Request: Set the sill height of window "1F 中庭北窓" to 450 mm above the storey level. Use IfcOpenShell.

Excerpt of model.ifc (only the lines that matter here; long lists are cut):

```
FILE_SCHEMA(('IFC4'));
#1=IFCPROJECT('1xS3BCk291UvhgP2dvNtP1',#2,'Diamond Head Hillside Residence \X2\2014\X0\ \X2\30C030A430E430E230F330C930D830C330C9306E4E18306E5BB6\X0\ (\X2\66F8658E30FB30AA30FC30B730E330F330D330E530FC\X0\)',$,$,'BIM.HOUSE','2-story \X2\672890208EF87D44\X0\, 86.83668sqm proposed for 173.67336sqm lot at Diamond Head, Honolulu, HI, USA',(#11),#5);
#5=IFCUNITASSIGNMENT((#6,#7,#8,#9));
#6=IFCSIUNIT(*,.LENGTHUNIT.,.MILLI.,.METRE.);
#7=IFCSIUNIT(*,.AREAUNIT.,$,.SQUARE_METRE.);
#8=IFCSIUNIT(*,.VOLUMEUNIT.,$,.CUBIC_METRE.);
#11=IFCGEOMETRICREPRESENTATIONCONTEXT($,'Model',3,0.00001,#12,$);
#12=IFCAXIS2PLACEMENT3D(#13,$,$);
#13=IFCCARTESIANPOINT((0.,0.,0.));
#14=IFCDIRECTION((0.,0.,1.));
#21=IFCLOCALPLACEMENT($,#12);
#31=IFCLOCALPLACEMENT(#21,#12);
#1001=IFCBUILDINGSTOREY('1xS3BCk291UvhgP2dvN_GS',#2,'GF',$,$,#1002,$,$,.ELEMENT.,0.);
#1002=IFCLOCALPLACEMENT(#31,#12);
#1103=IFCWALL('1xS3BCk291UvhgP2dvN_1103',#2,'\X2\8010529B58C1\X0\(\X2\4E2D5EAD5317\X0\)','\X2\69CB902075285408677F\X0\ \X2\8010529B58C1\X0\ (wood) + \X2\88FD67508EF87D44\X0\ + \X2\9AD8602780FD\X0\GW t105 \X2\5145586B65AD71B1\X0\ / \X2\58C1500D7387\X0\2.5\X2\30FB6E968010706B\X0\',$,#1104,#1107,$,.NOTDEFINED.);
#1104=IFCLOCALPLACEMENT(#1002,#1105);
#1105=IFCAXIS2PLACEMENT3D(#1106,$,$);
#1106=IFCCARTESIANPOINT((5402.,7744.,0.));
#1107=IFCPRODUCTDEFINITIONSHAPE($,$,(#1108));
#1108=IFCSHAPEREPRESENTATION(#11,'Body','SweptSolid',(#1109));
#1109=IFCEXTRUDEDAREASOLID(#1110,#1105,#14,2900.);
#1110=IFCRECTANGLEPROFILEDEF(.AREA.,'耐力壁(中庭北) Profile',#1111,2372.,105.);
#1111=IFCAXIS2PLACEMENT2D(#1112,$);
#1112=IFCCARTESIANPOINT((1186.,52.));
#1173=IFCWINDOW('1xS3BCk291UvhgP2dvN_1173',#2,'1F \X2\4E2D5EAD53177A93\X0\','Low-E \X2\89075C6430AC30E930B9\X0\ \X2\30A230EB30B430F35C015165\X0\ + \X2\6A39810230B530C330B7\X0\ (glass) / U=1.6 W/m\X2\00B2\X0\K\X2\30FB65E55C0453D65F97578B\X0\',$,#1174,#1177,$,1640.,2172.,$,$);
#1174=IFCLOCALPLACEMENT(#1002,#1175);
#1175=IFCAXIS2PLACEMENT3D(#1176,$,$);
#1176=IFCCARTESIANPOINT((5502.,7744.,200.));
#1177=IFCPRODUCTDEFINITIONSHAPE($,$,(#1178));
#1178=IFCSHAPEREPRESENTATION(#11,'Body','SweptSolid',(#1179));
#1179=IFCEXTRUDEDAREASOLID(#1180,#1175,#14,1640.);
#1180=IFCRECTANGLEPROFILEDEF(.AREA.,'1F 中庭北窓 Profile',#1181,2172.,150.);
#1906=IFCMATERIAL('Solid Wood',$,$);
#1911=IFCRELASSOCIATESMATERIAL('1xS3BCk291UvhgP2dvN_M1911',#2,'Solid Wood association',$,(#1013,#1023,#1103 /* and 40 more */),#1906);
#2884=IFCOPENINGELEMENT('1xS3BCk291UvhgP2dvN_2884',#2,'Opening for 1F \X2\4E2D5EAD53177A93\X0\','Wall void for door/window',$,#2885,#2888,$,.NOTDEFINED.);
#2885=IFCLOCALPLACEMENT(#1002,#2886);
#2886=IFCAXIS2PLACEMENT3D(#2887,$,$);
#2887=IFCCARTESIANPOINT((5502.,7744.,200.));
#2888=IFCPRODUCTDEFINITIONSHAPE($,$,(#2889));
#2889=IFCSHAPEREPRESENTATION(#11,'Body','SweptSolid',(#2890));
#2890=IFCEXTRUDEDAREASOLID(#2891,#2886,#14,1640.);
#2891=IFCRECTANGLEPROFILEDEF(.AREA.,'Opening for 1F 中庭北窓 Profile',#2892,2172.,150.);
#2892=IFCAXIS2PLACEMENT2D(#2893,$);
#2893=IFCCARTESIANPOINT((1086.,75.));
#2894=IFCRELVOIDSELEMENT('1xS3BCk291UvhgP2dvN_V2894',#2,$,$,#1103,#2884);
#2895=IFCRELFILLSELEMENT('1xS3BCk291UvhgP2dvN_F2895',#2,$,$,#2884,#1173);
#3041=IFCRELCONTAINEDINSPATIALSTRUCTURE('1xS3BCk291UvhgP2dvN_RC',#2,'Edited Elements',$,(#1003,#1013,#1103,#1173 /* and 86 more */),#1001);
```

```python
import numpy as np
import ifcopenshell
import ifcopenshell.api.geometry
import ifcopenshell.geom
import ifcopenshell.util.element
import ifcopenshell.util.placement
import ifcopenshell.util.shape
import ifcopenshell.util.unit

model = ifcopenshell.open("model.ifc")
unit_scale = ifcopenshell.util.unit.calculate_unit_scale(model)

window = model.by_guid("1xS3BCk291UvhgP2dvN_1173")
opening = window.FillsVoids[0].RelatingOpeningElement
storey = ifcopenshell.util.element.get_container(window, ifc_class="IfcBuildingStorey")
level = ifcopenshell.util.placement.get_local_placement(storey.ObjectPlacement)[2, 3]

# The opening's origin need not be at the sill, so measure its lowest point.
shape = ifcopenshell.geom.create_shape(ifcopenshell.geom.settings(), opening)
bottom = ifcopenshell.util.shape.get_shape_bottom_elevation(shape, shape.geometry) / unit_scale
dz = level + 450.0 - bottom

shift = np.array([0.0, 0.0, dz])
# The window is not placed relative to its opening, so move both.
for product in (opening, window):
    matrix = ifcopenshell.util.placement.get_local_placement(product.ObjectPlacement)
    matrix[:3, 3] += shift
    ifcopenshell.api.geometry.edit_object_placement(model, product=product, matrix=matrix, is_si=False)

print(f"moved by {dz * unit_scale:+.3f} m")

model.write("model_v2.ifc")
```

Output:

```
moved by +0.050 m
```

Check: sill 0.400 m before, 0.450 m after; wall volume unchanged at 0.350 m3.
